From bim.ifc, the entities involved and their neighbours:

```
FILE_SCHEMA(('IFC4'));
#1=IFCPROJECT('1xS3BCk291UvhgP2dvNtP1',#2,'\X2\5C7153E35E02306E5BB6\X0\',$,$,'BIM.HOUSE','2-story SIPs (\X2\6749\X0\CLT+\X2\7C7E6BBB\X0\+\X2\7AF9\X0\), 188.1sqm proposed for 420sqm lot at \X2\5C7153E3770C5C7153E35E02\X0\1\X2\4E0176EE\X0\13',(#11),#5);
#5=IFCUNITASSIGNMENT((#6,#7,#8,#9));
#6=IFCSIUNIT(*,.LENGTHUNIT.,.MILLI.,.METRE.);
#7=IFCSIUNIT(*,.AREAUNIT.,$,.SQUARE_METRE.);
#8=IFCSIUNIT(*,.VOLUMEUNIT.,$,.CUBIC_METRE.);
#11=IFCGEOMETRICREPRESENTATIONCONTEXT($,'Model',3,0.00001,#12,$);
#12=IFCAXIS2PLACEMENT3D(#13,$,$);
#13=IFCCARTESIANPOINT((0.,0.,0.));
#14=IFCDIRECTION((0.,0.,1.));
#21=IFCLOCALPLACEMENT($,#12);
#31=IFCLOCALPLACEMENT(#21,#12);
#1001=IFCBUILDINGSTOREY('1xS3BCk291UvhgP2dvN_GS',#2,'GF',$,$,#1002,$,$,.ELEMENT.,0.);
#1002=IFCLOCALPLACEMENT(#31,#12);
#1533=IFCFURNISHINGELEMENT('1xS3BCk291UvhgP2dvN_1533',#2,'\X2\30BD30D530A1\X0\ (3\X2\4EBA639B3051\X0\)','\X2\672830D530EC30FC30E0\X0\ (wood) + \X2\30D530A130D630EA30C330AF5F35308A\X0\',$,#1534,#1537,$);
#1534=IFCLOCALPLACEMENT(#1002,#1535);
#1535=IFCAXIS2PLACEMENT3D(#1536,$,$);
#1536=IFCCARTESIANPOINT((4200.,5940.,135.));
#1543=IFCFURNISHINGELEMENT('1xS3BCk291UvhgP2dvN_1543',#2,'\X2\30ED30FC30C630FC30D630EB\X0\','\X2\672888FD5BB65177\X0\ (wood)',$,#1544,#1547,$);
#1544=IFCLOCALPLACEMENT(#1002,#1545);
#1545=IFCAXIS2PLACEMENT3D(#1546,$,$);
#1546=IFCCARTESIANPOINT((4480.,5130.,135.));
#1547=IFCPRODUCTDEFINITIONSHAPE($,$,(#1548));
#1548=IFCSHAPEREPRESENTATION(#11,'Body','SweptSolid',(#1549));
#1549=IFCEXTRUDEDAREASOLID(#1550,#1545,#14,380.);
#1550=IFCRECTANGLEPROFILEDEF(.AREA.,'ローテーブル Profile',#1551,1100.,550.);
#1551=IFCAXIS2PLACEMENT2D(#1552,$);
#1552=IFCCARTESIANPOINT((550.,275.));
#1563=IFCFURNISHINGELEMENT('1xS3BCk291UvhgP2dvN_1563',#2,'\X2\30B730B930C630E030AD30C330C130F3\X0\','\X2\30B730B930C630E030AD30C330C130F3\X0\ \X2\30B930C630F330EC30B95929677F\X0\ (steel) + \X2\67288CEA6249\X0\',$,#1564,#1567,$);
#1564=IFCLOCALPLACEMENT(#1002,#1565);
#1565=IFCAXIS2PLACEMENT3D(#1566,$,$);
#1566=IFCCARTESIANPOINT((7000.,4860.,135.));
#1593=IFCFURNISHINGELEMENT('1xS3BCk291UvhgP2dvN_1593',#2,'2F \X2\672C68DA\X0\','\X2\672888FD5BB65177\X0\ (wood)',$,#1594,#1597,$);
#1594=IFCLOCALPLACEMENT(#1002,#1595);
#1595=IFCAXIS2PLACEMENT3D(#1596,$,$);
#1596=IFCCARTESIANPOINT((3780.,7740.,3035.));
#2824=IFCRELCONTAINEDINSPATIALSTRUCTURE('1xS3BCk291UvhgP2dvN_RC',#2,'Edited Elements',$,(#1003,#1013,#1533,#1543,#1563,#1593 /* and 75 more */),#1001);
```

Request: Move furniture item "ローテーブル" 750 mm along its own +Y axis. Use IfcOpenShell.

```python
import ifcopenshell
import ifcopenshell.api.geometry
import ifcopenshell.util.placement
import ifcopenshell.util.unit

model = ifcopenshell.open("bim.ifc")
unit_scale = ifcopenshell.util.unit.calculate_unit_scale(model)

item = model.by_guid("1xS3BCk291UvhgP2dvN_1543")
matrix = ifcopenshell.util.placement.get_local_placement(item.ObjectPlacement)
matrix[:3, 3] += matrix[:3, 1] * 0.75 / unit_scale
ifcopenshell.api.geometry.edit_object_placement(model, product=item, matrix=matrix, is_si=False)

print(ifcopenshell.util.placement.get_local_placement(item.ObjectPlacement).round(3) + 0.0)

model.write("bim_updated.ifc")
```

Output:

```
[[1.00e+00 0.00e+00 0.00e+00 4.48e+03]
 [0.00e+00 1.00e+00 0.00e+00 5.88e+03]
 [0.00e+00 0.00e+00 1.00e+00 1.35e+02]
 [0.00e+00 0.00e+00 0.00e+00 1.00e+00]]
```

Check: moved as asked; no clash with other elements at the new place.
